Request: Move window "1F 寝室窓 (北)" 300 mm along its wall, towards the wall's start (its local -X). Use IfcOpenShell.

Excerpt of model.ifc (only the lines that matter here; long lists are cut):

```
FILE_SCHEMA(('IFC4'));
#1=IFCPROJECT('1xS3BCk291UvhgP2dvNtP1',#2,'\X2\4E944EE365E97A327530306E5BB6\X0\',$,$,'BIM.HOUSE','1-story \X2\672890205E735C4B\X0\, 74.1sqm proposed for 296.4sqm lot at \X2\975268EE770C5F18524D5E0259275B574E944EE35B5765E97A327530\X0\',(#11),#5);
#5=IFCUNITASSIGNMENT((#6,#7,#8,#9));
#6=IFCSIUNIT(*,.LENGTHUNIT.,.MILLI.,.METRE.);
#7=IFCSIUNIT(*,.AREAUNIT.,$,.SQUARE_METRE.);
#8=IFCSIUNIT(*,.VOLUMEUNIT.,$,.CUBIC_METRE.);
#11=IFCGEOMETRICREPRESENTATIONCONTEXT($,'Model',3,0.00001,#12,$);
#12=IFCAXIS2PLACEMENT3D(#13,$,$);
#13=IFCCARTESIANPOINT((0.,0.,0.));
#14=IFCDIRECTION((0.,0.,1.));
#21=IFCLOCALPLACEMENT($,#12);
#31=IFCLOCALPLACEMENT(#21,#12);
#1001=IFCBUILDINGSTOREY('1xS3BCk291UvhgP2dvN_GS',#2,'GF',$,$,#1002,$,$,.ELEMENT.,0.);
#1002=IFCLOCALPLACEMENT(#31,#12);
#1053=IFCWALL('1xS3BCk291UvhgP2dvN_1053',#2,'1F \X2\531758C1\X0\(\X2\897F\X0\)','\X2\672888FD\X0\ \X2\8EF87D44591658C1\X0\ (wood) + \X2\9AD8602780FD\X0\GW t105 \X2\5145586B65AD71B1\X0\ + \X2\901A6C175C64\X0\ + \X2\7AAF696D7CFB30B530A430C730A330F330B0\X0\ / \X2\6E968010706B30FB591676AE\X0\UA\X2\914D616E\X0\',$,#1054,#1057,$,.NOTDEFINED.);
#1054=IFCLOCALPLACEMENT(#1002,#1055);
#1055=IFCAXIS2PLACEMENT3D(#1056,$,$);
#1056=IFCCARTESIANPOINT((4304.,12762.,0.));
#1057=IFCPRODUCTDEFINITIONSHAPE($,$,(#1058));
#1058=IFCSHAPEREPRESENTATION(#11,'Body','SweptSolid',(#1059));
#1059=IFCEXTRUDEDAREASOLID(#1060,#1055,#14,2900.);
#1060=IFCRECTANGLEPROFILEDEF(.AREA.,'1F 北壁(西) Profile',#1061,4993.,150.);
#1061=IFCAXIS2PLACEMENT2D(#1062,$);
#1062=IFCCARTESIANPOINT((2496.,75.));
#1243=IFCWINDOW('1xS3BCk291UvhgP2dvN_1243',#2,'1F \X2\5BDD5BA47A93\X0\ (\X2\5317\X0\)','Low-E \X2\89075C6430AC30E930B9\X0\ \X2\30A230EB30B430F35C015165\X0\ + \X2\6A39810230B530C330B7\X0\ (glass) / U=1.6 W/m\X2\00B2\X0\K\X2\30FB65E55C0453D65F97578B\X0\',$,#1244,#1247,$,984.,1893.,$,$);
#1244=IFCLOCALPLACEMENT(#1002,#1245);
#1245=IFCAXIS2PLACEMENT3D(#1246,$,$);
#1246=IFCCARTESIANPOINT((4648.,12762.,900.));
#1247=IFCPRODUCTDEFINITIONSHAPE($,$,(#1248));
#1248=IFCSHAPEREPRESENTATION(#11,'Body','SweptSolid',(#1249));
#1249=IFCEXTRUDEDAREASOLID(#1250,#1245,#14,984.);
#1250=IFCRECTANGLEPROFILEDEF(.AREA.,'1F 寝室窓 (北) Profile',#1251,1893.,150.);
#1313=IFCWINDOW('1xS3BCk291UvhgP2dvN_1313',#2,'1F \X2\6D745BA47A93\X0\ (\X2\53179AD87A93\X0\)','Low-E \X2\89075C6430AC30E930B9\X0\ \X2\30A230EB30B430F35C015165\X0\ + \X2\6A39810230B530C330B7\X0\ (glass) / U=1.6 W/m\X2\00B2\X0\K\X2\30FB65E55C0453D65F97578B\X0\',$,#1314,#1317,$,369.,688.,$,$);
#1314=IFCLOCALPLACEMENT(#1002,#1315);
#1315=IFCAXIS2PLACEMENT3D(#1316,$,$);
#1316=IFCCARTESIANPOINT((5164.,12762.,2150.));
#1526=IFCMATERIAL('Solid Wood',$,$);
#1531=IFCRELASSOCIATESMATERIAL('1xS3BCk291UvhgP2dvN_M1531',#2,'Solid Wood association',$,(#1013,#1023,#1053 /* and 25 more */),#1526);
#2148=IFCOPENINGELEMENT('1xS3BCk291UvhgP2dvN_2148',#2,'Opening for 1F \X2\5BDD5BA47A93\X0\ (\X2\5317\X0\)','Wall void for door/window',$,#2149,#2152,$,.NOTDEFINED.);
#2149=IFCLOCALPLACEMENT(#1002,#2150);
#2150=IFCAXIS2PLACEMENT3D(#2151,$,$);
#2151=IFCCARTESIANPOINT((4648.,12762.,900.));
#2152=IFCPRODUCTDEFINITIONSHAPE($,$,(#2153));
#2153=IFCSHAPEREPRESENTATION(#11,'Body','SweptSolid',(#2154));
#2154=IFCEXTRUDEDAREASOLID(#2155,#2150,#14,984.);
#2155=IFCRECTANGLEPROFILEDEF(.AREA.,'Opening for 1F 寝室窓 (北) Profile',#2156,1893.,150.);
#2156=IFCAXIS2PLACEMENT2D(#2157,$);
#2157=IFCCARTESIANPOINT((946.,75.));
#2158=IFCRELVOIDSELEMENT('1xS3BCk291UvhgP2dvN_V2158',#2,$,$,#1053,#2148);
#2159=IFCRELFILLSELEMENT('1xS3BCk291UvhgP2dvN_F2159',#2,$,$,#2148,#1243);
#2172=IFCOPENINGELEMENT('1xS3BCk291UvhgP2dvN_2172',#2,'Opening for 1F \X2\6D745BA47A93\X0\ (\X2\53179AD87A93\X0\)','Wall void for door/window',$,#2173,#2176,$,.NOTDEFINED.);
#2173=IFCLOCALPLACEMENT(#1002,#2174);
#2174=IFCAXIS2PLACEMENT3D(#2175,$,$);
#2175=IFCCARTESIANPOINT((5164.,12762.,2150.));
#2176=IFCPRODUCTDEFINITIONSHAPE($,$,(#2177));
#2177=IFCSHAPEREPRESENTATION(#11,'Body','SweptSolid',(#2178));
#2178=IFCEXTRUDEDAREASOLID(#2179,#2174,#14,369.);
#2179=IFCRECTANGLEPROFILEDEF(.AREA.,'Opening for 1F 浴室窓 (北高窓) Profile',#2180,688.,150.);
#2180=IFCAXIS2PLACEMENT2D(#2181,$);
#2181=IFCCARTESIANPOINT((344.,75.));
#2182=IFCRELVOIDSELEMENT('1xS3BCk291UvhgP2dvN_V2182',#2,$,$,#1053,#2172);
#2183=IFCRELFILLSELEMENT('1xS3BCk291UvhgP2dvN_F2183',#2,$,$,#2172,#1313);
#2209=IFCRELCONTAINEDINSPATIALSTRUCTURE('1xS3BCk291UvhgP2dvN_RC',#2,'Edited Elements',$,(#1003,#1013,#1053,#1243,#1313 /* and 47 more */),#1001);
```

```python
import ifcopenshell
import ifcopenshell.api.geometry
import ifcopenshell.util.placement

model = ifcopenshell.open("model.ifc")

window = model.by_guid("1xS3BCk291UvhgP2dvN_1243")
opening = window.FillsVoids[0].RelatingOpeningElement
wall = opening.VoidsElements[0].RelatingBuildingElement

wall_matrix = ifcopenshell.util.placement.get_local_placement(wall.ObjectPlacement)
shift = wall_matrix[:3, 0] * -300.0
before = ifcopenshell.util.placement.get_local_placement(window.ObjectPlacement)[:3, 3].copy()

# The window is not placed relative to its opening, so move both.
for product in (opening, window):
    matrix = ifcopenshell.util.placement.get_local_placement(product.ObjectPlacement)
    matrix[:3, 3] += shift
    ifcopenshell.api.geometry.edit_object_placement(model, product=product, matrix=matrix, is_si=False)

after = ifcopenshell.util.placement.get_local_placement(window.ObjectPlacement)[:3, 3]
print("window moved by", (after - before).round(3) + 0.0)

model.write("model_rev.ifc")
```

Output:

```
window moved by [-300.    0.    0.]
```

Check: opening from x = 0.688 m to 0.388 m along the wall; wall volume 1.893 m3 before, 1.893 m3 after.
